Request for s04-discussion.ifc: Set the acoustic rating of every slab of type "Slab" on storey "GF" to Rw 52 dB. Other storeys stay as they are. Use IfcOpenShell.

First a look at what the model holds.

```python
import ifcopenshell
import ifcopenshell.util.element

model = ifcopenshell.open("s04-discussion.ifc")
print(model.schema)
storey = next(s for s in model.by_type("IfcBuildingStorey") if s.Name == "GF")
slabs = [e for e in ifcopenshell.util.element.get_decomposition(storey) if e.is_a("IfcSlab")]
seen = {}
for e in slabs:
    element_type = ifcopenshell.util.element.get_type(e)
    key = (element_type.Name if element_type != e and element_type else None, ifcopenshell.util.element.get_pset(e, "Pset_SlabCommon", "AcousticRating"))
    seen[key] = seen.get(key, 0) + 1
for (name, value), count in sorted(seen.items(), key=str):
    print(count, "x", name, "|", value)
```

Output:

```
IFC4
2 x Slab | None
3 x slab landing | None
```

```python
import ifcopenshell
import ifcopenshell.api.pset
import ifcopenshell.util.element

model = ifcopenshell.open("s04-discussion.ifc")

storey = next(s for s in model.by_type("IfcBuildingStorey") if s.Name == "GF")
slabs = [e for e in ifcopenshell.util.element.get_decomposition(storey) if e.is_a("IfcSlab")]

count = 0
for e in slabs:
    element_type = ifcopenshell.util.element.get_type(e)
    if element_type in (None, e) or element_type.Name != "Slab":
        continue
    # add_pset returns the element's existing set when there is one.
    pset = ifcopenshell.api.pset.add_pset(model, product=e, name="Pset_SlabCommon")
    ifcopenshell.api.pset.edit_pset(model, pset=pset, properties={"AcousticRating": "Rw 52 dB"})
    count += 1

print(count, "slabs updated")

model.write("s04-discussion_rev.ifc")
```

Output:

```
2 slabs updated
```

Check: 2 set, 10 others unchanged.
